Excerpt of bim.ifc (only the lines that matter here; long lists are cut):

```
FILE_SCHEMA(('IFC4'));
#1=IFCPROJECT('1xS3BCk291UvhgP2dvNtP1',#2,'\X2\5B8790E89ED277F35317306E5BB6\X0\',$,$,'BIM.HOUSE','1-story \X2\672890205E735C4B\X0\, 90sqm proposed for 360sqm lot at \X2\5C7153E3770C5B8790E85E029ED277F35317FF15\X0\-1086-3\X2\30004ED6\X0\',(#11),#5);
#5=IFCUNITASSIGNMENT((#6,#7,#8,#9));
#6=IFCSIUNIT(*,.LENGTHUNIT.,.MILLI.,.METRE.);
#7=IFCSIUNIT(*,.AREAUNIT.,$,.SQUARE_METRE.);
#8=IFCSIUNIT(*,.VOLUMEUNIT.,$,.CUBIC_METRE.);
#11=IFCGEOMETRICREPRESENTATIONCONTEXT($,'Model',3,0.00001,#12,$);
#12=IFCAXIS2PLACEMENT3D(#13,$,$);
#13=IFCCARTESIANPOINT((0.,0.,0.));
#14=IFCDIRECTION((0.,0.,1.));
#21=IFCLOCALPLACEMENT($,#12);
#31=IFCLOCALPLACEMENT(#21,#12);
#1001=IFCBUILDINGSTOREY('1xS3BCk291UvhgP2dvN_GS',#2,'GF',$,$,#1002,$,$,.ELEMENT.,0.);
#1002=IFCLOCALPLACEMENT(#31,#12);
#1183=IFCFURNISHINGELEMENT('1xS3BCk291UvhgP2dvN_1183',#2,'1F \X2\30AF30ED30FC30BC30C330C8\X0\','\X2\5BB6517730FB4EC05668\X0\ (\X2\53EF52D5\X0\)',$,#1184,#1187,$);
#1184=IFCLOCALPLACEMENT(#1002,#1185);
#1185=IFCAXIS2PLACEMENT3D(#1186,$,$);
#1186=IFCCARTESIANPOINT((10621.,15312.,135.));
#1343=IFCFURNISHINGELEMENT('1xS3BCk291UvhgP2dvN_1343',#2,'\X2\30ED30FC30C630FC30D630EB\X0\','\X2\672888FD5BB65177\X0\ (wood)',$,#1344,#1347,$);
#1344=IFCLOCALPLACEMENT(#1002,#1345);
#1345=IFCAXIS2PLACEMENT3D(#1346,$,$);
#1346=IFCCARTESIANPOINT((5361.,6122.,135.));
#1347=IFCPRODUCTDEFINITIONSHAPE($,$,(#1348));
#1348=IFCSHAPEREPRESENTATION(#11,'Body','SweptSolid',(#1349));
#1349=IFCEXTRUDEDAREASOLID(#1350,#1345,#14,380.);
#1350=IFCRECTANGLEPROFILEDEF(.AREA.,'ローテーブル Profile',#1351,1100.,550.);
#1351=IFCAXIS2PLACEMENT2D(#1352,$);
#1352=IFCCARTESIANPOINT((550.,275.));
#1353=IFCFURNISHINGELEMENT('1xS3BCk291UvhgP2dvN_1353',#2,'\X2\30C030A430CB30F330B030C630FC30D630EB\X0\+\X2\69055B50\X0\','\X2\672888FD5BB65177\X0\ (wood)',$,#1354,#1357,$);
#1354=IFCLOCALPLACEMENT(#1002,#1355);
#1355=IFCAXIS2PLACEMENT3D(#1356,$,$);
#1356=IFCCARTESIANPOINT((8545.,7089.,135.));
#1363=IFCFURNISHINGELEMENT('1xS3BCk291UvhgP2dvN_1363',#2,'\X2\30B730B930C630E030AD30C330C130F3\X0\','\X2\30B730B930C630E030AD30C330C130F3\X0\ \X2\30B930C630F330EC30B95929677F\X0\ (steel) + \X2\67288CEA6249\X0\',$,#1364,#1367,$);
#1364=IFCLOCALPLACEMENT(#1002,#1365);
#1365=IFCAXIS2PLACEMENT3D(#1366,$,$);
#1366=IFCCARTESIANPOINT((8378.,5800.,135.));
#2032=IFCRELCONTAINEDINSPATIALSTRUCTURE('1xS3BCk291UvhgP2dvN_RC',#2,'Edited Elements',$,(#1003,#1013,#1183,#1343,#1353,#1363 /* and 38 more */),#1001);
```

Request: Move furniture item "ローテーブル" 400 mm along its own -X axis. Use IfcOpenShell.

```python
import ifcopenshell
import ifcopenshell.api.geometry
import ifcopenshell.util.placement

model = ifcopenshell.open("bim.ifc")

item = model.by_guid("1xS3BCk291UvhgP2dvN_1343")
matrix = ifcopenshell.util.placement.get_local_placement(item.ObjectPlacement)
matrix[:3, 3] -= matrix[:3, 0] * 400.0
ifcopenshell.api.geometry.edit_object_placement(model, product=item, matrix=matrix, is_si=False)

print(ifcopenshell.util.placement.get_local_placement(item.ObjectPlacement).round(3) + 0.0)

model.write("bim_edited.ifc")
```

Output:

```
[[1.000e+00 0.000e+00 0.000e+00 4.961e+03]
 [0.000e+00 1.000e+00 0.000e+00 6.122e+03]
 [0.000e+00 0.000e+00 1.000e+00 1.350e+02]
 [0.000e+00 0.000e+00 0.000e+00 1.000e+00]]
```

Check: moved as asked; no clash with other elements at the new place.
